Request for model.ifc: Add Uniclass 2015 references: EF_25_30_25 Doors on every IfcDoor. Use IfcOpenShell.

First a look at what the model holds.

```python
import ifcopenshell

model = ifcopenshell.open("model.ifc")
print(model.schema)
print("classifications:", [c.Name for c in model.by_type("IfcClassification")])
for ifc_class in ("IfcDoor", "IfcRoof", "IfcStair", "IfcWall", "IfcWindow"):
    print(ifc_class, len(model.by_type(ifc_class)))
```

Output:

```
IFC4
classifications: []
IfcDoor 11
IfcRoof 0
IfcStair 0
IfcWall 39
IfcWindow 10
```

```python
import ifcopenshell
import ifcopenshell.api.classification

model = ifcopenshell.open("model.ifc")

system = ifcopenshell.api.classification.add_classification(model, classification="Uniclass 2015")

codes = {
    "IfcDoor": ("EF_25_30_25", "Doors"),
}
for ifc_class, (code, name) in codes.items():
    products = model.by_type(ifc_class)
    ifcopenshell.api.classification.add_reference(
        model, products=products, classification=system, identification=code, name=name
    )
    print(code, len(products))

model.write("model-out.ifc")
```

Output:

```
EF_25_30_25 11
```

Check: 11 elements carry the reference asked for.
